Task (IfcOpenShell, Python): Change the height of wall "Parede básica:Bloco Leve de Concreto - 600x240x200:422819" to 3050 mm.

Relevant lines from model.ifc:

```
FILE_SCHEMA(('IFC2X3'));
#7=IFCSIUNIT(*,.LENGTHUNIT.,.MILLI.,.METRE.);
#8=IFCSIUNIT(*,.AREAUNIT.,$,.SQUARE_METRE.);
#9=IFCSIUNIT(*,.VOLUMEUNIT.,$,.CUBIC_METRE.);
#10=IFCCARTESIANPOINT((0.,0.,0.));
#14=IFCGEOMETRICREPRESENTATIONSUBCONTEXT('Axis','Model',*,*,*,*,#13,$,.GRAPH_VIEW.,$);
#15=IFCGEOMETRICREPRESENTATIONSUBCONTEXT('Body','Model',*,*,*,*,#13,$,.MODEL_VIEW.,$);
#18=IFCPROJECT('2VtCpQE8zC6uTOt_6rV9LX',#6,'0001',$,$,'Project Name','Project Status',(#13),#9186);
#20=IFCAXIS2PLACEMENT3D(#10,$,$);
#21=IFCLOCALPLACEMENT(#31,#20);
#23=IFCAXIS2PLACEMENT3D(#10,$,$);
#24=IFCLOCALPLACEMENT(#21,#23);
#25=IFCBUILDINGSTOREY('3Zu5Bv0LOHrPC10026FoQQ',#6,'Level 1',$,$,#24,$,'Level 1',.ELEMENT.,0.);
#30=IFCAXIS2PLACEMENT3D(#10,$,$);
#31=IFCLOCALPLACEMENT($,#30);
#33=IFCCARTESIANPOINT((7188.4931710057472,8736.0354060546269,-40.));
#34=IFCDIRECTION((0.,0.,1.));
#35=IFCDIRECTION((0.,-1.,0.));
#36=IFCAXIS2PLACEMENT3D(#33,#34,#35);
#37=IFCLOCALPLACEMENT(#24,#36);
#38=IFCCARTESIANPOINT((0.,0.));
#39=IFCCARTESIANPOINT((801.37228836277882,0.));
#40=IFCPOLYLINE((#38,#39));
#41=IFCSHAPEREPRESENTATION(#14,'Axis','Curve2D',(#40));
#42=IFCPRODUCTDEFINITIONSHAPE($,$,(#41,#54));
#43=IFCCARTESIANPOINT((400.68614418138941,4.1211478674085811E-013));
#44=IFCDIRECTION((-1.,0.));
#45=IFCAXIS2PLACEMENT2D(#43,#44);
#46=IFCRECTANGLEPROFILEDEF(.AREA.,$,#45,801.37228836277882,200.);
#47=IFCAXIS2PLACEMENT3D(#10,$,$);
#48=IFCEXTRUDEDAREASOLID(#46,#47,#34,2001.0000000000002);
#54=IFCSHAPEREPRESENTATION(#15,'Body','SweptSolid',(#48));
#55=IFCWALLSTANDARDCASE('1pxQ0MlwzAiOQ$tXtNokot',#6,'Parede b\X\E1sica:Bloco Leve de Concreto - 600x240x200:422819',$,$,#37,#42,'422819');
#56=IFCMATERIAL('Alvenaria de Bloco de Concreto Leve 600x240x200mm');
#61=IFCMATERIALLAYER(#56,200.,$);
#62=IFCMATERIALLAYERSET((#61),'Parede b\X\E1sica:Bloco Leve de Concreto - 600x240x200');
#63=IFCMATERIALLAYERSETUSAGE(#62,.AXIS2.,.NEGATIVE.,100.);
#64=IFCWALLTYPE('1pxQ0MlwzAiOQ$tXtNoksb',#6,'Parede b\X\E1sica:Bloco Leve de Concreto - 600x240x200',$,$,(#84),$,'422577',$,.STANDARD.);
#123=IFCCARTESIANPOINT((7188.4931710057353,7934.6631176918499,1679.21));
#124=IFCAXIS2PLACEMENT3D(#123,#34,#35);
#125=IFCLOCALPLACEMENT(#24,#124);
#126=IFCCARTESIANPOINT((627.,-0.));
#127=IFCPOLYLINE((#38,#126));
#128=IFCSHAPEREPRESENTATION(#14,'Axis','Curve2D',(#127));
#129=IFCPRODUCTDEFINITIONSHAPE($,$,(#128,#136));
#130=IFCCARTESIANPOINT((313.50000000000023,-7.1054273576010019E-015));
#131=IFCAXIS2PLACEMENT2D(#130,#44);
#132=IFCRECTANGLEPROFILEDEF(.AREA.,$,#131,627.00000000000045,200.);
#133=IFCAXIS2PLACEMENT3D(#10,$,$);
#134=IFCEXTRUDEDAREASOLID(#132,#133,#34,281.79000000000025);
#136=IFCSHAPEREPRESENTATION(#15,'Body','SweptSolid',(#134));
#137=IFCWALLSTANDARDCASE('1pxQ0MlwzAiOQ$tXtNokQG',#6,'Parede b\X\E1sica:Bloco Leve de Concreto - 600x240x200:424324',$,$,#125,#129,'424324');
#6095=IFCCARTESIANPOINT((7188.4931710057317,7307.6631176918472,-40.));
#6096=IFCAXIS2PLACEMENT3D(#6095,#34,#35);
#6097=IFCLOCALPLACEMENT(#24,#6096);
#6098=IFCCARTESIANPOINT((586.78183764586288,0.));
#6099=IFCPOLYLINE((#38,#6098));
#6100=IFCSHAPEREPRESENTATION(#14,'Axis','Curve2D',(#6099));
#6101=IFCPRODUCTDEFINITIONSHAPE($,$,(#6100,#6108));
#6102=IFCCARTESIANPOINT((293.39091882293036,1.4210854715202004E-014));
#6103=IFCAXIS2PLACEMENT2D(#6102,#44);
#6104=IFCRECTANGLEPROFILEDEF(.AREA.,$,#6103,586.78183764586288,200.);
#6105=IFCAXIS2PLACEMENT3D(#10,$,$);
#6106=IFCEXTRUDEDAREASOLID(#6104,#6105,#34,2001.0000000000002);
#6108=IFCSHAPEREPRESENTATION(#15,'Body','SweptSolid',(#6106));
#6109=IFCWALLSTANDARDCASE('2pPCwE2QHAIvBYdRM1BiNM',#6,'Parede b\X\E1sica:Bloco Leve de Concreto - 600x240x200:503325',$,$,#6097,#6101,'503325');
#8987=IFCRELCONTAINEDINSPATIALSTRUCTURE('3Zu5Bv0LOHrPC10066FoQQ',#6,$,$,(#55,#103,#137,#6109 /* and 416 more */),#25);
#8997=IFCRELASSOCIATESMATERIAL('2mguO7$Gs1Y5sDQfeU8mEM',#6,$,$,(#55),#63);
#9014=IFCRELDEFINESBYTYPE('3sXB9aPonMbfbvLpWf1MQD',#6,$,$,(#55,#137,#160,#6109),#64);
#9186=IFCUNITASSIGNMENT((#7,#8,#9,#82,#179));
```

```python
import ifcopenshell
import ifcopenshell.geom
import ifcopenshell.util.representation
import ifcopenshell.util.shape
import ifcopenshell.util.unit

model = ifcopenshell.open("model.ifc")
unit_scale = ifcopenshell.util.unit.calculate_unit_scale(model)
settings = ifcopenshell.geom.settings()


def volume(element):
    """Net volume in cubic metres, openings subtracted."""
    shape = ifcopenshell.geom.create_shape(settings, element)
    return ifcopenshell.util.shape.get_volume(shape.geometry)


wall = model.by_guid("1pxQ0MlwzAiOQ$tXtNokot")
before = volume(wall)

body = ifcopenshell.util.representation.get_representation(wall, "Model", "Body")
solid = body.Items[0]
old_height = solid.Depth
solid.Depth = 3.05 / unit_scale
after = volume(wall)

print(f"height {old_height:g} -> {solid.Depth:g}, volume {before:.3f} -> {after:.3f} m3")

model.write("model-out.ifc")
```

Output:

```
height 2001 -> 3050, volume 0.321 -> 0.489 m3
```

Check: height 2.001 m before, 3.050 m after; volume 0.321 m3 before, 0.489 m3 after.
